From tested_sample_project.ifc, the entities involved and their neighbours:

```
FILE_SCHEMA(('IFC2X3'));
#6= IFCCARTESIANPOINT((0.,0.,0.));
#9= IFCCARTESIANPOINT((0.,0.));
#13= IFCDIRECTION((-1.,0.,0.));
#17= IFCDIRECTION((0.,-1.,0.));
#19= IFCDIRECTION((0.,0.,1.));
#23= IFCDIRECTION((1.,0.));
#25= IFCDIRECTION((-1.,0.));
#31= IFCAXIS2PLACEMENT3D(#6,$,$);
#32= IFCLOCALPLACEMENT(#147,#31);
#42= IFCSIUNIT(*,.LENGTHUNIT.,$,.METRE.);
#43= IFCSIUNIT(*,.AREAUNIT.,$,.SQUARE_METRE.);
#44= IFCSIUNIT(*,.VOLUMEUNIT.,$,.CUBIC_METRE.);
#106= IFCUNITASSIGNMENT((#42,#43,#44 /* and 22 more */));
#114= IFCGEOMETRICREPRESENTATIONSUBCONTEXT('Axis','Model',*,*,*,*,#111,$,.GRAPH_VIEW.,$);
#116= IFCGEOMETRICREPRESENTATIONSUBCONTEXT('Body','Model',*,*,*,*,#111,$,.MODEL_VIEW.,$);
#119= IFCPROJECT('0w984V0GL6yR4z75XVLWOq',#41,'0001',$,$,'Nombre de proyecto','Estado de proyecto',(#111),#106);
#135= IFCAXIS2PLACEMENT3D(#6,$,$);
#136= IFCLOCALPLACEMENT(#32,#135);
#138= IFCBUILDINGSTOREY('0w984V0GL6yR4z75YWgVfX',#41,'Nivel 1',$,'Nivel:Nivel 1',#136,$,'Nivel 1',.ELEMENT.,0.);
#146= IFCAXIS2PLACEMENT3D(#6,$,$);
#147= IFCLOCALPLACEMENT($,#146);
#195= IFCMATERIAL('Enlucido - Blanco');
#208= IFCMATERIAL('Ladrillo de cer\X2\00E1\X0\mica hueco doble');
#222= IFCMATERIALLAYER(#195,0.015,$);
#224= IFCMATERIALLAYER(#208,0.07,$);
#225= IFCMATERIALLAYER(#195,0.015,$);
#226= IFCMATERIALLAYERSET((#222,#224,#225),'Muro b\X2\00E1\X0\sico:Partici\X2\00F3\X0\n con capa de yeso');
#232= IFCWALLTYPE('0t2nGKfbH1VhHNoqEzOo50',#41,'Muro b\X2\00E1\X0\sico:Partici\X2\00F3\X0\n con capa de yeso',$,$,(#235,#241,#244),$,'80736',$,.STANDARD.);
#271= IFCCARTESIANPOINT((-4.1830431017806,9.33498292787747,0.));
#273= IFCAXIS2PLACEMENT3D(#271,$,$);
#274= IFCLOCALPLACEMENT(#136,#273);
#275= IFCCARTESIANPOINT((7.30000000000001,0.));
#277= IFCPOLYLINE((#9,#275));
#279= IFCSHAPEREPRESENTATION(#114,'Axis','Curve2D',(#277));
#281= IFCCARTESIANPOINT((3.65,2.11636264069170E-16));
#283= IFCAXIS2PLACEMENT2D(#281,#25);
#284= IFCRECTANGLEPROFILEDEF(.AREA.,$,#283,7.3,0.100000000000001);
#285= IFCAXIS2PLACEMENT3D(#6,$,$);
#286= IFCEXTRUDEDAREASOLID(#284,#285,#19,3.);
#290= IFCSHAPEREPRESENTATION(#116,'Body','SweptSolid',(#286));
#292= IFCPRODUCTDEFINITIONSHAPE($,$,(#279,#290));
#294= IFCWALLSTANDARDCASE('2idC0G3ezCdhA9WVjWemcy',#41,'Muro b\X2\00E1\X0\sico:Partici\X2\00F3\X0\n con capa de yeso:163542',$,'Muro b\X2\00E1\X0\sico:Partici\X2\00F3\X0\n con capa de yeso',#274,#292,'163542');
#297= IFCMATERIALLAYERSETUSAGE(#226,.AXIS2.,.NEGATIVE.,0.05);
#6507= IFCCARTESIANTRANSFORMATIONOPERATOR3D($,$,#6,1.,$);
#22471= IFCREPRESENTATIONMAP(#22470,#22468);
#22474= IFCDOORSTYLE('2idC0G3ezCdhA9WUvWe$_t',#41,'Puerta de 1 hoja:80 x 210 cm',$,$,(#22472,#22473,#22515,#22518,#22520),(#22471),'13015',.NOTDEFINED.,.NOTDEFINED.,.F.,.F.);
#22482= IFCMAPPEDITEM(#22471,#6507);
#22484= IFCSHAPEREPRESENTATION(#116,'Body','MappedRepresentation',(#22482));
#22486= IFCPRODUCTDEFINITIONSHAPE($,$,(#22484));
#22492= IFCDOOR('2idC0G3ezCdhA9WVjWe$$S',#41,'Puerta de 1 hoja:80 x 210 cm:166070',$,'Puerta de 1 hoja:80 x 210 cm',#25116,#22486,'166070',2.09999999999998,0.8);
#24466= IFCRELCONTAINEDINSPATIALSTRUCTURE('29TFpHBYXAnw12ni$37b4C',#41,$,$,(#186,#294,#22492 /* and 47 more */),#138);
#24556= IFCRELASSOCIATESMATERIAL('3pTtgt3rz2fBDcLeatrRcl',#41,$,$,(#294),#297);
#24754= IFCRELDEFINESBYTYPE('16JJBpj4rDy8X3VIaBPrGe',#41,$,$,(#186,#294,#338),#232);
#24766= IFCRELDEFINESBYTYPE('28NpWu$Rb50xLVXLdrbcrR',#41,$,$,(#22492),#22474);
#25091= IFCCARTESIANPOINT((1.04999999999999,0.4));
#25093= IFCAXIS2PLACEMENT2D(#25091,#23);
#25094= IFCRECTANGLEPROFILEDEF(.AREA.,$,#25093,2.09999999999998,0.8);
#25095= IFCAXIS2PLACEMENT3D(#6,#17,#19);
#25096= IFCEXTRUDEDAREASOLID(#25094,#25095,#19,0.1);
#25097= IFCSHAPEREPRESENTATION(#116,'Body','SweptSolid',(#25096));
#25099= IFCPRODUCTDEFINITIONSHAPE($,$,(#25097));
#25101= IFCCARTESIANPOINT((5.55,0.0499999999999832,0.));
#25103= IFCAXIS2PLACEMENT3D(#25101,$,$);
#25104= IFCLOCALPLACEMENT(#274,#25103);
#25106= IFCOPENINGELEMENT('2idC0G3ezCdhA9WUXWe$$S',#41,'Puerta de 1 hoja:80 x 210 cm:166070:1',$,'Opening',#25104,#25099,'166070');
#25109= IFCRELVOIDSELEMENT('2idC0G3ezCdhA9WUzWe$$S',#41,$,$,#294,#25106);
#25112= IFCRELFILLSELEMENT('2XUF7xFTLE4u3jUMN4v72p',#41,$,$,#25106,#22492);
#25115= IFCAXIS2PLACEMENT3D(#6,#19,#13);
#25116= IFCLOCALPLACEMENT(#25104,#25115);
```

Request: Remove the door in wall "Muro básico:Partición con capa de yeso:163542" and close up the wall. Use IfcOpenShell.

```python
import ifcopenshell
import ifcopenshell.api.feature
import ifcopenshell.api.root
import ifcopenshell.geom
import ifcopenshell.util.shape

model = ifcopenshell.open("tested_sample_project.ifc")
settings = ifcopenshell.geom.settings()


def volume(element):
    """Net volume in cubic metres, openings subtracted."""
    shape = ifcopenshell.geom.create_shape(settings, element)
    return ifcopenshell.util.shape.get_volume(shape.geometry)


door = model.by_guid("2idC0G3ezCdhA9WVjWe$$S")
opening = door.FillsVoids[0].RelatingOpeningElement
wall = opening.VoidsElements[0].RelatingBuildingElement
before = volume(wall)

ifcopenshell.api.root.remove_product(model, product=door)
ifcopenshell.api.feature.remove_feature(model, feature=opening)

after = volume(wall)

print(f"wall volume {before:.3f} -> {after:.3f} m3")

model.write("tested_sample_project_updated.ifc")
```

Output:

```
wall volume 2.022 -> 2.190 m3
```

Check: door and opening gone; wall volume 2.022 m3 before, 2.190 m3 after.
